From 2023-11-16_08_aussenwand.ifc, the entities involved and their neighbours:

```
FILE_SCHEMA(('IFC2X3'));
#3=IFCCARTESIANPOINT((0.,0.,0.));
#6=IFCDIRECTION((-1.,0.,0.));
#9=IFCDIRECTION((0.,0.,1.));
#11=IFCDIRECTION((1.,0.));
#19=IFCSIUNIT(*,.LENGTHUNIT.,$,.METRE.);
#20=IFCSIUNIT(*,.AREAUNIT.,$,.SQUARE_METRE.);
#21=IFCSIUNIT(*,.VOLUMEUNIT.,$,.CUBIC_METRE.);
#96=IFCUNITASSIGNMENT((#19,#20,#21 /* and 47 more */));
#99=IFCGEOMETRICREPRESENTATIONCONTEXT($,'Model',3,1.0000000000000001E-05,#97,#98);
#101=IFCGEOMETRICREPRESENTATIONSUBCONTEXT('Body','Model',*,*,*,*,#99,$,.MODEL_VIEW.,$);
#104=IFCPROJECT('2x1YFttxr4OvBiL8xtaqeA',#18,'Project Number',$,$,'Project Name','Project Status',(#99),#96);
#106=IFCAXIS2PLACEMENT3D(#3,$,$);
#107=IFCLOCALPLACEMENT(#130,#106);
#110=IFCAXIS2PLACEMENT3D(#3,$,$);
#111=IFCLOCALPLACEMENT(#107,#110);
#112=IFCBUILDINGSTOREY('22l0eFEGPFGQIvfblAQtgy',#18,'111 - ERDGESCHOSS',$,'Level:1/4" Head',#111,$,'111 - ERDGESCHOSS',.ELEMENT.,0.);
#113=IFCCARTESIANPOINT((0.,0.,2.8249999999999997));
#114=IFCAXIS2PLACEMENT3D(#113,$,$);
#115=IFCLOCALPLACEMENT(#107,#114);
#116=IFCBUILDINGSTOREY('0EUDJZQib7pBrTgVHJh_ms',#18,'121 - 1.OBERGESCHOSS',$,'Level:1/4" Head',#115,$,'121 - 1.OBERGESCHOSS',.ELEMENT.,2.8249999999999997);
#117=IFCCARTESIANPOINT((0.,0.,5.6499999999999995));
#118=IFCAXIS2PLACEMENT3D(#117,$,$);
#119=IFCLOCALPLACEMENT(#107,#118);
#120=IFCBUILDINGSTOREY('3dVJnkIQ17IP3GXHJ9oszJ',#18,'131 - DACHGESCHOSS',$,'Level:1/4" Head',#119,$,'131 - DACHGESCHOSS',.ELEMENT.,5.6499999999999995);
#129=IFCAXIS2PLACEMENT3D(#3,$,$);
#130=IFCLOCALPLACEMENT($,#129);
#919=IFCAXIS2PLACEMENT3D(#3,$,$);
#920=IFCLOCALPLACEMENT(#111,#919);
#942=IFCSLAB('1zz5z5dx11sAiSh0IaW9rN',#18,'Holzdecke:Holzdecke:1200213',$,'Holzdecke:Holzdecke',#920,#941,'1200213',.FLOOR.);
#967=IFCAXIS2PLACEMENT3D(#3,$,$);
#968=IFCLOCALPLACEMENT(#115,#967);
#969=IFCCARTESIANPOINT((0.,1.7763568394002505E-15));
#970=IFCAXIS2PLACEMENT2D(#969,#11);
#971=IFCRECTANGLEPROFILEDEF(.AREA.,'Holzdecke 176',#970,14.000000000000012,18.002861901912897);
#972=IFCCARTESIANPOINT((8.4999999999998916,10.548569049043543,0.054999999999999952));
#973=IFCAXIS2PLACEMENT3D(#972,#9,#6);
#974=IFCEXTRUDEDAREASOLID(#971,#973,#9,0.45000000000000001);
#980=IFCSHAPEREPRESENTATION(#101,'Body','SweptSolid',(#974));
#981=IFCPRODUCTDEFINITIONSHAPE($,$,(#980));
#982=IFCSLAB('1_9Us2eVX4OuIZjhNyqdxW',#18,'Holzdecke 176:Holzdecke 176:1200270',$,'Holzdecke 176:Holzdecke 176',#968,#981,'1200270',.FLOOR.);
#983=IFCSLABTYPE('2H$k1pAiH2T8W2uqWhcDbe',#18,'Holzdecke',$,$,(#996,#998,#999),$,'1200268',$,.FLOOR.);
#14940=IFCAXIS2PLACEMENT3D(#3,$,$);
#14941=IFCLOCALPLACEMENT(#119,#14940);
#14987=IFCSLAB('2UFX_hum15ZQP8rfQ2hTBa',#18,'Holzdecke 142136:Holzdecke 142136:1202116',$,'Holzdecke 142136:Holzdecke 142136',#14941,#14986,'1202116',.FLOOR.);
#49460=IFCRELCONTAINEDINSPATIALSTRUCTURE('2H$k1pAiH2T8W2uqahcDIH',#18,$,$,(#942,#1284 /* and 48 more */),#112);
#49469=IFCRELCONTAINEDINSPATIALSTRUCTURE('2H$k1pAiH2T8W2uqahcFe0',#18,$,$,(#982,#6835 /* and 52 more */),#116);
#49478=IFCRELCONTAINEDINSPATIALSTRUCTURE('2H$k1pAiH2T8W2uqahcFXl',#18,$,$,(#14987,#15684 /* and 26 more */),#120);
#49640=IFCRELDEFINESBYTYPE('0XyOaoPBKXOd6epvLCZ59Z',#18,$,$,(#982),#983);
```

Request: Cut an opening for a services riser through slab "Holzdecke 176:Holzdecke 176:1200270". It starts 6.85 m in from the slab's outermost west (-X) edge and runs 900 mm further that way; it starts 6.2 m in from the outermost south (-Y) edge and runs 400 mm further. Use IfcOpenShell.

```python
import numpy as np
import ifcopenshell
import ifcopenshell.api.feature
import ifcopenshell.api.geometry
import ifcopenshell.api.root
import ifcopenshell.geom
import ifcopenshell.util.placement
import ifcopenshell.util.representation
import ifcopenshell.util.shape
import ifcopenshell.util.unit

model = ifcopenshell.open("2023-11-16_08_aussenwand.ifc")
unit_scale = ifcopenshell.util.unit.calculate_unit_scale(model)
settings = ifcopenshell.geom.settings()


def volume(element):
    """Net volume in cubic metres, openings subtracted."""
    shape = ifcopenshell.geom.create_shape(settings, element)
    return ifcopenshell.util.shape.get_volume(shape.geometry)


slab = model.by_guid("1_9Us2eVX4OuIZjhNyqdxW")
before = volume(slab)

# Extent in the slab's own axes, in metres. The edges named are its -X and -Y sides.
slab_shape = ifcopenshell.geom.create_shape(settings, slab)
vertices = ifcopenshell.util.shape.get_vertices(slab_shape.geometry)
x_min, y_min, bottom = vertices.min(axis=0)
top = vertices[:, 2].max()

opening = ifcopenshell.api.root.create_entity(model, ifc_class="IfcOpeningElement", name="Services riser opening")
context = ifcopenshell.util.representation.get_context(model, "Model", "Body", "MODEL_VIEW")
width, depth = 0.9, 0.4
outline = [(0.0, 0.0), (width, 0.0), (width, depth), (0.0, depth), (0.0, 0.0)]
# Overshoot both faces by 50 mm so the cut is clean.
shape = ifcopenshell.api.geometry.add_slab_representation(
    model, context=context, depth=top - bottom + 0.1, polyline=outline
)
ifcopenshell.api.geometry.assign_representation(model, product=opening, representation=shape)

matrix = ifcopenshell.util.placement.get_local_placement(slab.ObjectPlacement)
matrix[:, 3] = matrix @ np.append(np.array([x_min + 6.85, y_min + 6.2, bottom - 0.05]) / unit_scale, 1.0)
ifcopenshell.api.geometry.edit_object_placement(model, product=opening, matrix=matrix, is_si=False)
ifcopenshell.api.feature.add_feature(model, feature=opening, element=slab)

after = volume(slab)

print(f"slab volume {before:.3f} -> {after:.3f} m3")

model.write("2023-11-16_08_aussenwand-out.ifc")
```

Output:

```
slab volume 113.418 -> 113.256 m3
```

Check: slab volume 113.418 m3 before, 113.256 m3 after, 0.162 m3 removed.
